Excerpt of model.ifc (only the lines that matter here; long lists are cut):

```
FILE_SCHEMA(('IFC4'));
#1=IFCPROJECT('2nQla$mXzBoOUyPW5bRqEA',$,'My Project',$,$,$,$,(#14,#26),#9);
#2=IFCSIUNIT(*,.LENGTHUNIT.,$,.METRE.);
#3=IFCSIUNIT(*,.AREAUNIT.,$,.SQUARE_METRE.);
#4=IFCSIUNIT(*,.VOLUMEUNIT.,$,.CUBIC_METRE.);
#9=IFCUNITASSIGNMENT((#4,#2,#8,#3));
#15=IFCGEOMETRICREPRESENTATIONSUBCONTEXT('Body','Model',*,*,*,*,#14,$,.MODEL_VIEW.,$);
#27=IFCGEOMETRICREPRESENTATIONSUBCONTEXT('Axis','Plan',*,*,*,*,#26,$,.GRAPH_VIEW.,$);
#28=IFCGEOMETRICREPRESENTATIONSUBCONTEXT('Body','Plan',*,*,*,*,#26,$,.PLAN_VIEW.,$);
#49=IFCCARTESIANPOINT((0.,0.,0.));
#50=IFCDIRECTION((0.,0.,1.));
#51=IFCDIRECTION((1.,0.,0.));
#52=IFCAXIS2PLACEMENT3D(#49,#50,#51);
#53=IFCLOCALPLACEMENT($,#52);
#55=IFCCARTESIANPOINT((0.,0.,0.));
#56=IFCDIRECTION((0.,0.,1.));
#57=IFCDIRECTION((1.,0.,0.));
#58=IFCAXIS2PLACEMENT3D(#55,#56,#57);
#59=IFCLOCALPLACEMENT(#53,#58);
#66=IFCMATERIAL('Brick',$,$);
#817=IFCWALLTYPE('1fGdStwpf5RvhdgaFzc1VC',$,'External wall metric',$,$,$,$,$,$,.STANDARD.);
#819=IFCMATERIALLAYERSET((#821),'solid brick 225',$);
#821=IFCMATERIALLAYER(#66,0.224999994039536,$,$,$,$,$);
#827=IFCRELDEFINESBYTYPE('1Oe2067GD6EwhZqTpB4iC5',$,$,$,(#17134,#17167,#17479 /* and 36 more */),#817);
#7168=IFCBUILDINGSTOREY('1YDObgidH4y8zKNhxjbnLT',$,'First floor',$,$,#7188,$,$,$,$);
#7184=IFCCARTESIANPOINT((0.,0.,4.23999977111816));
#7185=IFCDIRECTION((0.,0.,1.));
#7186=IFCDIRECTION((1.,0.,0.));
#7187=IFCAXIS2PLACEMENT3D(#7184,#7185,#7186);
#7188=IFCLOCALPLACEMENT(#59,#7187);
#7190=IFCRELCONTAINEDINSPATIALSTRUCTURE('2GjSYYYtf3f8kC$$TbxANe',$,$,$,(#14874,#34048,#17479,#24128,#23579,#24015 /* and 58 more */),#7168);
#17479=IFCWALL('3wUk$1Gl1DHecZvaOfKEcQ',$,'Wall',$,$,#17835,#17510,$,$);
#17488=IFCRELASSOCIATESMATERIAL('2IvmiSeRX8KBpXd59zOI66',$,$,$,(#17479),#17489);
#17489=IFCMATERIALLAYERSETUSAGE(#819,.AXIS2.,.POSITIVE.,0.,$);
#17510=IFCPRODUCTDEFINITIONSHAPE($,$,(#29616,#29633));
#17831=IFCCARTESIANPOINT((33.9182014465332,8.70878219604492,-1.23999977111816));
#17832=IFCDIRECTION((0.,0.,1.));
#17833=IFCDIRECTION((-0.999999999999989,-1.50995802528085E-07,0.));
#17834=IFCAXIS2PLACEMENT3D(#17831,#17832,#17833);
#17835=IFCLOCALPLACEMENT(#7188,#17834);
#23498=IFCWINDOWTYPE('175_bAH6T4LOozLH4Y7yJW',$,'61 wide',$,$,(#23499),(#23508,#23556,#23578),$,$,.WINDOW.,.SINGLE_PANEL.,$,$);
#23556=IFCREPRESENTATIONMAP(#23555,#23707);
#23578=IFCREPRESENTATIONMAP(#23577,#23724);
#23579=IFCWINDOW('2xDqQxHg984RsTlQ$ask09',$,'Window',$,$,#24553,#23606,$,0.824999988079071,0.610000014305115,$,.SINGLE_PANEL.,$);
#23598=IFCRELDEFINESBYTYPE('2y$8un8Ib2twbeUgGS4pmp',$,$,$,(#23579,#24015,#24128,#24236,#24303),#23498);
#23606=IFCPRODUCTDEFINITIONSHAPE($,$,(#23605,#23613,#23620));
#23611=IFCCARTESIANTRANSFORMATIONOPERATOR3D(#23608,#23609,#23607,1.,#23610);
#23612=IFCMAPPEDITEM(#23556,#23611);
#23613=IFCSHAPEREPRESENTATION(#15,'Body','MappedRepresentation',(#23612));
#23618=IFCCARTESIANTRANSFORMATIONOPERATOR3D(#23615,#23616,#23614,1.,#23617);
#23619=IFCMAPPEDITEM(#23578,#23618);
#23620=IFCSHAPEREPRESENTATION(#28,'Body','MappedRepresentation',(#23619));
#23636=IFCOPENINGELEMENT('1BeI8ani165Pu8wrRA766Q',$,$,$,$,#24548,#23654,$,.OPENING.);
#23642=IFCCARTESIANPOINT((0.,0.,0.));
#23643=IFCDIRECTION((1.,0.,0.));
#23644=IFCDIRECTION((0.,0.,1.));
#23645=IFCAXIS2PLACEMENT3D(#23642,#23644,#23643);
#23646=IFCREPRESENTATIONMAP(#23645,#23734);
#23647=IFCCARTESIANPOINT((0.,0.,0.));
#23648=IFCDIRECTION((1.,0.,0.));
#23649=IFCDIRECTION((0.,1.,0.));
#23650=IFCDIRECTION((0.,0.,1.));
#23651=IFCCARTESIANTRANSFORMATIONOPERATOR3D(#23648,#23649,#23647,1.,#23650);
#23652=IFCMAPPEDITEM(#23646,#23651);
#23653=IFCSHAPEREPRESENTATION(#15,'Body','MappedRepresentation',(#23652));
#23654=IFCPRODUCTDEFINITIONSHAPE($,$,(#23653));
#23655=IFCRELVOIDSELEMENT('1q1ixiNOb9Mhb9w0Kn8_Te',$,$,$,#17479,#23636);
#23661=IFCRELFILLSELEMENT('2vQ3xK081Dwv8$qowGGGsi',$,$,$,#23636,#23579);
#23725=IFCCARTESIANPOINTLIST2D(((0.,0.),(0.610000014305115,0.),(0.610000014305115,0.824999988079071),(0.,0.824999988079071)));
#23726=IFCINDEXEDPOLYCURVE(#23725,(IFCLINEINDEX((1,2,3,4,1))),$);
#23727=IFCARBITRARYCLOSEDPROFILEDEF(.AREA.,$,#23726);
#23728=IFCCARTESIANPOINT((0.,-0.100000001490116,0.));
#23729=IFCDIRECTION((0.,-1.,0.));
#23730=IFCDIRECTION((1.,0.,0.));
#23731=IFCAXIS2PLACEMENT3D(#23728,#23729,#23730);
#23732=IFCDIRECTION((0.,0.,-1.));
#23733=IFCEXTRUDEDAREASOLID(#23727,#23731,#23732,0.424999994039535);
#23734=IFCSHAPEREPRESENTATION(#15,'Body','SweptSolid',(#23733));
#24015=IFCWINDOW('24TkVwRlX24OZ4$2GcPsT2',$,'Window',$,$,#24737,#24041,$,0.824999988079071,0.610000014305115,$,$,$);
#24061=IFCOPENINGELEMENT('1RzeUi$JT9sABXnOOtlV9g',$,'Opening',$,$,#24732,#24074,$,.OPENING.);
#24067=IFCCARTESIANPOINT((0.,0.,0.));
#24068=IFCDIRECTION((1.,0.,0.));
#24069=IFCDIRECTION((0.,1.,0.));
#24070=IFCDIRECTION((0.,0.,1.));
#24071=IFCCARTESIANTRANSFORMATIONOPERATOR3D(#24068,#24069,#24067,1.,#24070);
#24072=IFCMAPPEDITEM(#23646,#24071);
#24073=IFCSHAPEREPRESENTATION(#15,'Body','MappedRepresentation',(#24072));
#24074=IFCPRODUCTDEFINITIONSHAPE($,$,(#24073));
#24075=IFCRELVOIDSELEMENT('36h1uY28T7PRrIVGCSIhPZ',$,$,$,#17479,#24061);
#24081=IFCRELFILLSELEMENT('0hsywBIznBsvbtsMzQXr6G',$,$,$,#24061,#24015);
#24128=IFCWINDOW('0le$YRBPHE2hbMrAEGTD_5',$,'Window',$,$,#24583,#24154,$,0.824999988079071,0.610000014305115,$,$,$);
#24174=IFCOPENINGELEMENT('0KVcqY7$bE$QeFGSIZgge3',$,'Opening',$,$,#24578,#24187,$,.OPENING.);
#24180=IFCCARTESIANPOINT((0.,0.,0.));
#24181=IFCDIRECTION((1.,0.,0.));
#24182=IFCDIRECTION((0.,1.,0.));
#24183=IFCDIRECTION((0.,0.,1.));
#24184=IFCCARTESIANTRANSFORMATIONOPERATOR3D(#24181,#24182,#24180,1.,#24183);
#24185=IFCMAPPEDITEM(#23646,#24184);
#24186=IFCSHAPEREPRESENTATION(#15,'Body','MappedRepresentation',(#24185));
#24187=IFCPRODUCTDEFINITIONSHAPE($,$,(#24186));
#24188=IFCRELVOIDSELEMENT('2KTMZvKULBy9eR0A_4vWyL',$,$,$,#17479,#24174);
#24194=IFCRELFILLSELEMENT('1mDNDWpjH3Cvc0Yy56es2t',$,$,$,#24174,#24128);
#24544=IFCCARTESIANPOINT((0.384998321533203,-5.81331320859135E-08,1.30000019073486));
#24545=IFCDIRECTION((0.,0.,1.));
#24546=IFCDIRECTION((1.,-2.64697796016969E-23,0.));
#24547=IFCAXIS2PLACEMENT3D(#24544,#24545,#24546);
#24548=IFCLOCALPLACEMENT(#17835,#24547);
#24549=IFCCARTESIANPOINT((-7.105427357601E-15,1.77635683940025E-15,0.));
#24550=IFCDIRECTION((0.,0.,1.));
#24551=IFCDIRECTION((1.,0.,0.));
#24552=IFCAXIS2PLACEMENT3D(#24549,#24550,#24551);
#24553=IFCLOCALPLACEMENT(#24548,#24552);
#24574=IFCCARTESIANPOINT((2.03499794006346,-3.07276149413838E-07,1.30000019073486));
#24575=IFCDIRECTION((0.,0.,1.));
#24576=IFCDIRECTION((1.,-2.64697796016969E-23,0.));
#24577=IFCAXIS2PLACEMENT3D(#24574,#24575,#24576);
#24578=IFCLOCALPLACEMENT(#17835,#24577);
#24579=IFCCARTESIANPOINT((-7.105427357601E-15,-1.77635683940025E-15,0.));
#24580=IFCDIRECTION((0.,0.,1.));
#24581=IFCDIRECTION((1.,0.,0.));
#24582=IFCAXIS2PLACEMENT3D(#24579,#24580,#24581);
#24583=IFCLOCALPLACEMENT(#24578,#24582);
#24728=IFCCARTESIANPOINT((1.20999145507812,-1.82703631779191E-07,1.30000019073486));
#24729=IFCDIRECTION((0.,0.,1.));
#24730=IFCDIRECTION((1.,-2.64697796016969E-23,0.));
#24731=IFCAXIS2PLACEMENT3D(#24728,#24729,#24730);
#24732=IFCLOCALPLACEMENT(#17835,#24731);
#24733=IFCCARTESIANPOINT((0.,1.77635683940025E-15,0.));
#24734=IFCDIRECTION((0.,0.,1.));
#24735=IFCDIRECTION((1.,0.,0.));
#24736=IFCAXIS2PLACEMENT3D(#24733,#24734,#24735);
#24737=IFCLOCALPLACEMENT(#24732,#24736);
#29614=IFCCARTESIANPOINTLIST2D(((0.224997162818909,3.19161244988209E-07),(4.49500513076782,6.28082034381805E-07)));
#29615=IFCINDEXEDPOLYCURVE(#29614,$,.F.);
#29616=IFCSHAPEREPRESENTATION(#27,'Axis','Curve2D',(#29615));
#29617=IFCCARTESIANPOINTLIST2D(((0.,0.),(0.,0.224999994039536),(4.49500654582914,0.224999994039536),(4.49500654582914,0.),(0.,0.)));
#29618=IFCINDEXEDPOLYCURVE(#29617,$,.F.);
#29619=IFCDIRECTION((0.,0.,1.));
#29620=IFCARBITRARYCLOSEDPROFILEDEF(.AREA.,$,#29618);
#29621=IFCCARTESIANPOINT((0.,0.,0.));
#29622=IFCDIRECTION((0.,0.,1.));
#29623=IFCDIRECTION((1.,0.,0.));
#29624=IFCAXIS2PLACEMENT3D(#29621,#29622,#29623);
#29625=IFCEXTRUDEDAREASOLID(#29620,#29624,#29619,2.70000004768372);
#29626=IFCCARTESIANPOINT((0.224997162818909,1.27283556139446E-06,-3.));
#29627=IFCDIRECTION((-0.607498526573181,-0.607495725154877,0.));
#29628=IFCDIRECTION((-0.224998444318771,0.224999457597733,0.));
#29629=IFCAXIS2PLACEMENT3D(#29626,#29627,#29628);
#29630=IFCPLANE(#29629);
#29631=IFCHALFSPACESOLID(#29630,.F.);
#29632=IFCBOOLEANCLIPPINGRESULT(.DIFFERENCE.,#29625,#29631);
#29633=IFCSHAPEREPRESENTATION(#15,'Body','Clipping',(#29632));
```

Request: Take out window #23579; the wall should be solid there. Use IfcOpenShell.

```python
import ifcopenshell
import ifcopenshell.api.feature
import ifcopenshell.api.root
import ifcopenshell.geom
import ifcopenshell.util.shape

model = ifcopenshell.open("model.ifc")
settings = ifcopenshell.geom.settings()


def volume(element):
    """Net volume in cubic metres, openings subtracted."""
    shape = ifcopenshell.geom.create_shape(settings, element)
    return ifcopenshell.util.shape.get_volume(shape.geometry)


window = model.by_guid("2xDqQxHg984RsTlQ$ask09")
opening = window.FillsVoids[0].RelatingOpeningElement
wall = opening.VoidsElements[0].RelatingBuildingElement
before = volume(wall)

ifcopenshell.api.root.remove_product(model, product=window)
ifcopenshell.api.feature.remove_feature(model, feature=opening)

after = volume(wall)

print(f"wall volume {before:.3f} -> {after:.3f} m3")

model.write("model_updated.ifc")
```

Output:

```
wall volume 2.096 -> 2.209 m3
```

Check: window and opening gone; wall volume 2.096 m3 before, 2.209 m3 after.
